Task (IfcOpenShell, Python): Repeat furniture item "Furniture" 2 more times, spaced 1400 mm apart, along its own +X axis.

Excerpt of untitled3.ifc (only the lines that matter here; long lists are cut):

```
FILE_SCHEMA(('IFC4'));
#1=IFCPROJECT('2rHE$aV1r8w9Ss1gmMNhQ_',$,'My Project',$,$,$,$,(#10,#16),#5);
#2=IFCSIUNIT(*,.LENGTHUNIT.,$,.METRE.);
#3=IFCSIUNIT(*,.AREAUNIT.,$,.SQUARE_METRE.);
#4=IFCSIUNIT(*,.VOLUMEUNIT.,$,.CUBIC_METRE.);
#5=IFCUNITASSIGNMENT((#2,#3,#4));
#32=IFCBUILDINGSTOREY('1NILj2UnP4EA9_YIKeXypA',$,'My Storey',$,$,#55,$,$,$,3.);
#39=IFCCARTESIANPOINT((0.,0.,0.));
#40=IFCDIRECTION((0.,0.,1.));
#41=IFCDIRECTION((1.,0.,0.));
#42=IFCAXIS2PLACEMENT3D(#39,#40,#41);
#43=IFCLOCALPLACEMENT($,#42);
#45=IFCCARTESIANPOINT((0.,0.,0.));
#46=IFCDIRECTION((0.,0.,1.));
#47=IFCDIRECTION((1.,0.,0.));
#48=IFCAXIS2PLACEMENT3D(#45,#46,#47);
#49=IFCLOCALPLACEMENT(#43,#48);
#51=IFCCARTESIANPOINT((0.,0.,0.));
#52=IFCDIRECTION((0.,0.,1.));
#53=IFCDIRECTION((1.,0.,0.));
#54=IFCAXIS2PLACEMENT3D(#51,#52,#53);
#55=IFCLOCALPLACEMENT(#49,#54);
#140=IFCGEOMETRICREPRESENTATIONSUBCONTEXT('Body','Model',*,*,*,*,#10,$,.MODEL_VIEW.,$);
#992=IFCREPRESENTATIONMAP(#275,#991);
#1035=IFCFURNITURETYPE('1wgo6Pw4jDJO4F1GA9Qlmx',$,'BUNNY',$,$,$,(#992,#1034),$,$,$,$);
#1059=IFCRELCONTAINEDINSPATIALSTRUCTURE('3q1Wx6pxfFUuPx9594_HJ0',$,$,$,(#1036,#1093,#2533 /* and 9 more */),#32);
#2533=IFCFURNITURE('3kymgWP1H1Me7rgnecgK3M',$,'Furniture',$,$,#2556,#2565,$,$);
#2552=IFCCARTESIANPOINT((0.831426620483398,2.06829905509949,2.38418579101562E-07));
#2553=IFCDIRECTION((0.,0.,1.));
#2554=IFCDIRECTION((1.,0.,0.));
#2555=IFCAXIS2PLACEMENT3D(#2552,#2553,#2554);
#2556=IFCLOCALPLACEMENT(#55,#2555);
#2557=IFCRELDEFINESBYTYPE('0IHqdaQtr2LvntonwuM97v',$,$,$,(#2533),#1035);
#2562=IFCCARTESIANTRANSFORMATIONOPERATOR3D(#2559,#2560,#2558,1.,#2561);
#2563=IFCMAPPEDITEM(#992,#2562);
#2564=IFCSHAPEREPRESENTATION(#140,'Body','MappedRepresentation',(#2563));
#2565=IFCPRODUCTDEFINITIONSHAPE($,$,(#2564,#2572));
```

```python
import ifcopenshell
import ifcopenshell.api.geometry
import ifcopenshell.api.root
import ifcopenshell.util.element
import ifcopenshell.util.placement

model = ifcopenshell.open("untitled3.ifc")

source = model.by_guid("3kymgWP1H1Me7rgnecgK3M")
base = ifcopenshell.util.placement.get_local_placement(source.ObjectPlacement)
step = base[:3, 0] * 1.4

for i in range(1, 3):
    copy = ifcopenshell.api.root.copy_class(model, product=source)
    copy.Representation = ifcopenshell.util.element.copy_deep(
        model, source.Representation, exclude=["IfcGeometricRepresentationContext", "IfcRepresentationMap"]
    )
    matrix = base.copy()
    matrix[:3, 3] += i * step
    print("added at", matrix[:3, 3].round(3) + 0.0)
    ifcopenshell.api.geometry.edit_object_placement(model, product=copy, matrix=matrix, is_si=False)

model.write("untitled3_updated.ifc")
```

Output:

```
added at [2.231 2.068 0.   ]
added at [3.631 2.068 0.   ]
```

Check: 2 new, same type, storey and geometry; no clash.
